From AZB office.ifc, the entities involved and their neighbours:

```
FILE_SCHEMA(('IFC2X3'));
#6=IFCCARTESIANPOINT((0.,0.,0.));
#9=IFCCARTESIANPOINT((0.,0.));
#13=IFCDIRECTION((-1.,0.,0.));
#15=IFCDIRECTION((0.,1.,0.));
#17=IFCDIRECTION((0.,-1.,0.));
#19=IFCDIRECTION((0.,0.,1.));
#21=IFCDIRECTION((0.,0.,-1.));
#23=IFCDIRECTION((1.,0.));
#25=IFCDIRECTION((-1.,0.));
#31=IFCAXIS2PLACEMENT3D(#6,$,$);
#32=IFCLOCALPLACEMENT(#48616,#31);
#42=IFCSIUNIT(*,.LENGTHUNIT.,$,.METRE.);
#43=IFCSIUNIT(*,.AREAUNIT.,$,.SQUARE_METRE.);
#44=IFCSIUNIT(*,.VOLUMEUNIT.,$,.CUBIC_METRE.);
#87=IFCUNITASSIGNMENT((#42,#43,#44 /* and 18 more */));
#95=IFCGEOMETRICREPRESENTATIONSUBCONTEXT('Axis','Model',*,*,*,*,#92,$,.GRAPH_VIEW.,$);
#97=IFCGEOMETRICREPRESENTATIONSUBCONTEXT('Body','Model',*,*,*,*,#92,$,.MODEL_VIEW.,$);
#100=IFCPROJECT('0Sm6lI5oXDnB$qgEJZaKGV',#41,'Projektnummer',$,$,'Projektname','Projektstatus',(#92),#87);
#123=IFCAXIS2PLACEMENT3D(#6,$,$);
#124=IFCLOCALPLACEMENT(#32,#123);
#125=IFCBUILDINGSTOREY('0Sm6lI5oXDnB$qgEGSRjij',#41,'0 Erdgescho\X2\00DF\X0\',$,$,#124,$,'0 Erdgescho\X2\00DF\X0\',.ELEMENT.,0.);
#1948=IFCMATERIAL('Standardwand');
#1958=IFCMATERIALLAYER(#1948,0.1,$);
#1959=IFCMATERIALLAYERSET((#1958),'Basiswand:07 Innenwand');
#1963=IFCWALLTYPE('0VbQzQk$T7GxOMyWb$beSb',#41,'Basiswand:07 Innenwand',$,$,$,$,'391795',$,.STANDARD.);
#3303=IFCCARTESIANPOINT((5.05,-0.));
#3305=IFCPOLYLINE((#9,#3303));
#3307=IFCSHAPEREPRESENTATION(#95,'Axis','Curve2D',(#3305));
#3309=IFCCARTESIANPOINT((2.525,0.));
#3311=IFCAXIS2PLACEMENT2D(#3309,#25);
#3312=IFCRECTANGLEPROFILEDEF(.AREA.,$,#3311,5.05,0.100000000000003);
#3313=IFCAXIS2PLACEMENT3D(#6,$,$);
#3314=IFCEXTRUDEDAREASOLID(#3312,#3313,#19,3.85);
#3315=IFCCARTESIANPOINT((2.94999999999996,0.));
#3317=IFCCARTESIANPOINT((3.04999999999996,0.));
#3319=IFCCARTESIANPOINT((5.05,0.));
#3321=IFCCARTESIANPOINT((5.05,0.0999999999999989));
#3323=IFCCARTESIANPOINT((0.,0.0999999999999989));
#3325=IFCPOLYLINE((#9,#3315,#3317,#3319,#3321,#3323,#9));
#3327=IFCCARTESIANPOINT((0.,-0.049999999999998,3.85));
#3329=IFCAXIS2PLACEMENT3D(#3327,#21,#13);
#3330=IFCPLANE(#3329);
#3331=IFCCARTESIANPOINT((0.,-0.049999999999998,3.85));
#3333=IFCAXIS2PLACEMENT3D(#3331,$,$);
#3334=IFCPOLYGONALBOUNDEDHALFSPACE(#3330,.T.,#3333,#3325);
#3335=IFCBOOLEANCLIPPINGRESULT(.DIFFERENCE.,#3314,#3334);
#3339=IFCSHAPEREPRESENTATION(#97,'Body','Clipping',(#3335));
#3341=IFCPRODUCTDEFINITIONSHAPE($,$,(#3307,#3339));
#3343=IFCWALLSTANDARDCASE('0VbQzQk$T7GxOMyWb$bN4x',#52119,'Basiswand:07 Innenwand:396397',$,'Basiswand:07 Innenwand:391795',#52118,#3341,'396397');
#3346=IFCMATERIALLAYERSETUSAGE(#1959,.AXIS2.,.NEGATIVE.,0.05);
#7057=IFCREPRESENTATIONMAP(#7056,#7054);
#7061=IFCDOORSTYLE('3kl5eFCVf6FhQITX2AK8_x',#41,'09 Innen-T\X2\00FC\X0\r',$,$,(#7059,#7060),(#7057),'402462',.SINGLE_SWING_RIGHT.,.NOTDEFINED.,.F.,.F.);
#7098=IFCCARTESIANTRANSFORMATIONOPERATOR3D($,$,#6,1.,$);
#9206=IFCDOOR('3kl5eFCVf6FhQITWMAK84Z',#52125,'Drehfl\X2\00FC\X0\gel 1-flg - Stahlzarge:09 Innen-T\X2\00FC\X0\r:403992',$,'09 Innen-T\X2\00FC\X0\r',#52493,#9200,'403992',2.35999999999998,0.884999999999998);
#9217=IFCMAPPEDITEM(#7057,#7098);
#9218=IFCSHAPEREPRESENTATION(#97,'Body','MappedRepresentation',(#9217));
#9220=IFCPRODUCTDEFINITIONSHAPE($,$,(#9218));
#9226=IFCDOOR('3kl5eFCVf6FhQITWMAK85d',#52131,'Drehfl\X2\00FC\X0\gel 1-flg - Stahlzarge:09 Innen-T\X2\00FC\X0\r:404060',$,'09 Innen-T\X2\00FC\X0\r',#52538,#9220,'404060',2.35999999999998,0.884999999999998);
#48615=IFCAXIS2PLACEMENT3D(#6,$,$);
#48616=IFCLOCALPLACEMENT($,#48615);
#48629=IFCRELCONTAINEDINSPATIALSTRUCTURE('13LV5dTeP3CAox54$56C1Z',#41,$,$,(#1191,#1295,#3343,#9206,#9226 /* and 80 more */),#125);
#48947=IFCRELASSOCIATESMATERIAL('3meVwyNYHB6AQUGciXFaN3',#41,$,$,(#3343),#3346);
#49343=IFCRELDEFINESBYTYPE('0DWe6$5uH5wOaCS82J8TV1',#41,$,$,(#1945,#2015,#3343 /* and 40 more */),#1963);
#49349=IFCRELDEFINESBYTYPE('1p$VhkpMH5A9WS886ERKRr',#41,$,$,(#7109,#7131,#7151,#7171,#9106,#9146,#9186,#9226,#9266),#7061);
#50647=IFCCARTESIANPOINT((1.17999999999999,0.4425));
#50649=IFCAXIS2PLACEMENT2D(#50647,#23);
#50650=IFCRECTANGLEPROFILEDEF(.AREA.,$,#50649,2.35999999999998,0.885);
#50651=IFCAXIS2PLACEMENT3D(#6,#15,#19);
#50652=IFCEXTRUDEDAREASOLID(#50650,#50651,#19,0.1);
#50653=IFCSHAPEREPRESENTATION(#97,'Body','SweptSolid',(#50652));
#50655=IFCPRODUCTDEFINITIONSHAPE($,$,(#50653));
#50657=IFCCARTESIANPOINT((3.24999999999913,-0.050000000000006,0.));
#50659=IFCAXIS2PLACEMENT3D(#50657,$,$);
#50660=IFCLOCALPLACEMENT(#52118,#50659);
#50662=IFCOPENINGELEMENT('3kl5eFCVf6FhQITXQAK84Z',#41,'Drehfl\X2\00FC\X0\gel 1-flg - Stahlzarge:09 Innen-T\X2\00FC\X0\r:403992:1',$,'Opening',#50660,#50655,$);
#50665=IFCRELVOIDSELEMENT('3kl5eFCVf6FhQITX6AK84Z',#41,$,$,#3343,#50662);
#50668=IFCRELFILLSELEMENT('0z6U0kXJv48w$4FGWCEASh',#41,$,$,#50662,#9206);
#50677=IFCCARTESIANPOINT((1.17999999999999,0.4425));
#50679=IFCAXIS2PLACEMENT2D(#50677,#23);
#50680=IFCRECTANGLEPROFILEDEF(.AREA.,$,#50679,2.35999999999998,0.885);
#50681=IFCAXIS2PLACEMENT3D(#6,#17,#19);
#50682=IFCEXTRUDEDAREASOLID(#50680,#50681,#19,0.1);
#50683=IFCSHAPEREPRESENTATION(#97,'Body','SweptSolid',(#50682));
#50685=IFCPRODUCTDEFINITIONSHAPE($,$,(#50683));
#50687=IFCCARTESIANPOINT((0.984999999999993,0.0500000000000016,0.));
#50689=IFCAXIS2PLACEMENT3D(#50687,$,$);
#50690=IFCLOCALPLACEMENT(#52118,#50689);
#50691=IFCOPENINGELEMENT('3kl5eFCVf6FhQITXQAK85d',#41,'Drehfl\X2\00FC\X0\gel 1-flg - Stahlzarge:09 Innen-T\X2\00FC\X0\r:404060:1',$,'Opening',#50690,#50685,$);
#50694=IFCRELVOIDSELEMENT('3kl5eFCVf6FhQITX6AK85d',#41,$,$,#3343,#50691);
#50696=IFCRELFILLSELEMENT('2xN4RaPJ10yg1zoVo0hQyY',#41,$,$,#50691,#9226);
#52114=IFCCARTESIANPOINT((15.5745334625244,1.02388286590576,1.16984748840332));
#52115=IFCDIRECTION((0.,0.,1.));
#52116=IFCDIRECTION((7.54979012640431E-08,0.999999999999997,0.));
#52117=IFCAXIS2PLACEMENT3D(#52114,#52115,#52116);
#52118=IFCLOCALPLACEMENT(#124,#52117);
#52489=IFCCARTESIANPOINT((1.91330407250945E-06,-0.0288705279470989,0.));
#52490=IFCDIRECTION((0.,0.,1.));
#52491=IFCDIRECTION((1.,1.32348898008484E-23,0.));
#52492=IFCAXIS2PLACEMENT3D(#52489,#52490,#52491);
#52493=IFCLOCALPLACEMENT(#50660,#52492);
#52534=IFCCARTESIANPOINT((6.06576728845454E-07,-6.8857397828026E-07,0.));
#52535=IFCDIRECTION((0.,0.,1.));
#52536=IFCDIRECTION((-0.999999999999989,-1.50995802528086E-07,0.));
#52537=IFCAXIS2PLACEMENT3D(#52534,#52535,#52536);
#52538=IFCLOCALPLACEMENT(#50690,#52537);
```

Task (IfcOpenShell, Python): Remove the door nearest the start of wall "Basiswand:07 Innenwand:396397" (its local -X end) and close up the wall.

```python
import ifcopenshell
import ifcopenshell.api.feature
import ifcopenshell.api.root
import ifcopenshell.geom
import ifcopenshell.util.shape

model = ifcopenshell.open("AZB office.ifc")
settings = ifcopenshell.geom.settings()


def volume(element):
    """Net volume in cubic metres, openings subtracted."""
    shape = ifcopenshell.geom.create_shape(settings, element)
    return ifcopenshell.util.shape.get_volume(shape.geometry)


door = model.by_guid("3kl5eFCVf6FhQITWMAK85d")
opening = door.FillsVoids[0].RelatingOpeningElement
wall = opening.VoidsElements[0].RelatingBuildingElement
before = volume(wall)

ifcopenshell.api.root.remove_product(model, product=door)
ifcopenshell.api.feature.remove_feature(model, feature=opening)

after = volume(wall)

print(f"wall volume {before:.3f} -> {after:.3f} m3")

model.write("AZB office_rev.ifc")
```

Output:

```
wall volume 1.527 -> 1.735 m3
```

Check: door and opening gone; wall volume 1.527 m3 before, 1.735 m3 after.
